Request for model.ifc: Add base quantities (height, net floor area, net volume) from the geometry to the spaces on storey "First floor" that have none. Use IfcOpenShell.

First a look at what the model holds.

```python
import ifcopenshell
import ifcopenshell.util.element
import ifcopenshell.util.unit

model = ifcopenshell.open("model.ifc")
print(model.schema)
for unit_type in ("LENGTHUNIT", "AREAUNIT", "VOLUMEUNIT"):
    print(unit_type, ifcopenshell.util.unit.calculate_unit_scale(model, unit_type))
storey = next(s for s in model.by_type("IfcBuildingStorey") if s.Name == "First floor")
spaces = [e for e in ifcopenshell.util.element.get_decomposition(storey) if e.is_a("IfcSpace")]
for e in sorted(spaces, key=lambda e: e.id()):
    print(e.id(), e.is_a(), e.Name, list(ifcopenshell.util.element.get_psets(e, qtos_only=True)), sep=" | ")
```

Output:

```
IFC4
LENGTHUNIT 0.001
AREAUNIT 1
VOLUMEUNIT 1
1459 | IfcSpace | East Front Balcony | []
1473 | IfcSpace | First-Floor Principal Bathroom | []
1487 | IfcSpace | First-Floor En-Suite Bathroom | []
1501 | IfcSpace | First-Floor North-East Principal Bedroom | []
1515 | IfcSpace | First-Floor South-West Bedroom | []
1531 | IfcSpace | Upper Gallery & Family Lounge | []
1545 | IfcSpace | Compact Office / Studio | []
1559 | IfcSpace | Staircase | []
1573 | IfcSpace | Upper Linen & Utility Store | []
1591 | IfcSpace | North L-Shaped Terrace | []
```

```python
import ifcopenshell
import ifcopenshell.api.pset
import ifcopenshell.geom
import ifcopenshell.util.element
import ifcopenshell.util.shape
import ifcopenshell.util.unit

model = ifcopenshell.open("model.ifc")
unit_scale = ifcopenshell.util.unit.calculate_unit_scale(model)
area_scale = ifcopenshell.util.unit.calculate_unit_scale(model, "AREAUNIT")
volume_scale = ifcopenshell.util.unit.calculate_unit_scale(model, "VOLUMEUNIT")
settings = ifcopenshell.geom.settings()

storey = next(s for s in model.by_type("IfcBuildingStorey") if s.Name == "First floor")
spaces = [e for e in ifcopenshell.util.element.get_decomposition(storey) if e.is_a("IfcSpace")]

for e in sorted(spaces, key=lambda e: e.id()):
    if ifcopenshell.util.element.get_psets(e, qtos_only=True, should_inherit=False):
        continue
    # Geometry comes back in metres, in the element's own axes.
    shape = ifcopenshell.geom.create_shape(settings, e)
    values = {
        "Height": ifcopenshell.util.shape.get_z(shape.geometry) / unit_scale,
        "NetFloorArea": ifcopenshell.util.shape.get_footprint_area(shape.geometry) / area_scale,
        "NetVolume": ifcopenshell.util.shape.get_volume(shape.geometry) / volume_scale,
    }
    qto = ifcopenshell.api.pset.add_qto(model, product=e, name="Qto_SpaceBaseQuantities")
    ifcopenshell.api.pset.edit_qto(model, qto=qto, properties=values)
    print(e.id(), {k: round(v, 3) for k, v in values.items()})

model.write("model-out.ifc")
```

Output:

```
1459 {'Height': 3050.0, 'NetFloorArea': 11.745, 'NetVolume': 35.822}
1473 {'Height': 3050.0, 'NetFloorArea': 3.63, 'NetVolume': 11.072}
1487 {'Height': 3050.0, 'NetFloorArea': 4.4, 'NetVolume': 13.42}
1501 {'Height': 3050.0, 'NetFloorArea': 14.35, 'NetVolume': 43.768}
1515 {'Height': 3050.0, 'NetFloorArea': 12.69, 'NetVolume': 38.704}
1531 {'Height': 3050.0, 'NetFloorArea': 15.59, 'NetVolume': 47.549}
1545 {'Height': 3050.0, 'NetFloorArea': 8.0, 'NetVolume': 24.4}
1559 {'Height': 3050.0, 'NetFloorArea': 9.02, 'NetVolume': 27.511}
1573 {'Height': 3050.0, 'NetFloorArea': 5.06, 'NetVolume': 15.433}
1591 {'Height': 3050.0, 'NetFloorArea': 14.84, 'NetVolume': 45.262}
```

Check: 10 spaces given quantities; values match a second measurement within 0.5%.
